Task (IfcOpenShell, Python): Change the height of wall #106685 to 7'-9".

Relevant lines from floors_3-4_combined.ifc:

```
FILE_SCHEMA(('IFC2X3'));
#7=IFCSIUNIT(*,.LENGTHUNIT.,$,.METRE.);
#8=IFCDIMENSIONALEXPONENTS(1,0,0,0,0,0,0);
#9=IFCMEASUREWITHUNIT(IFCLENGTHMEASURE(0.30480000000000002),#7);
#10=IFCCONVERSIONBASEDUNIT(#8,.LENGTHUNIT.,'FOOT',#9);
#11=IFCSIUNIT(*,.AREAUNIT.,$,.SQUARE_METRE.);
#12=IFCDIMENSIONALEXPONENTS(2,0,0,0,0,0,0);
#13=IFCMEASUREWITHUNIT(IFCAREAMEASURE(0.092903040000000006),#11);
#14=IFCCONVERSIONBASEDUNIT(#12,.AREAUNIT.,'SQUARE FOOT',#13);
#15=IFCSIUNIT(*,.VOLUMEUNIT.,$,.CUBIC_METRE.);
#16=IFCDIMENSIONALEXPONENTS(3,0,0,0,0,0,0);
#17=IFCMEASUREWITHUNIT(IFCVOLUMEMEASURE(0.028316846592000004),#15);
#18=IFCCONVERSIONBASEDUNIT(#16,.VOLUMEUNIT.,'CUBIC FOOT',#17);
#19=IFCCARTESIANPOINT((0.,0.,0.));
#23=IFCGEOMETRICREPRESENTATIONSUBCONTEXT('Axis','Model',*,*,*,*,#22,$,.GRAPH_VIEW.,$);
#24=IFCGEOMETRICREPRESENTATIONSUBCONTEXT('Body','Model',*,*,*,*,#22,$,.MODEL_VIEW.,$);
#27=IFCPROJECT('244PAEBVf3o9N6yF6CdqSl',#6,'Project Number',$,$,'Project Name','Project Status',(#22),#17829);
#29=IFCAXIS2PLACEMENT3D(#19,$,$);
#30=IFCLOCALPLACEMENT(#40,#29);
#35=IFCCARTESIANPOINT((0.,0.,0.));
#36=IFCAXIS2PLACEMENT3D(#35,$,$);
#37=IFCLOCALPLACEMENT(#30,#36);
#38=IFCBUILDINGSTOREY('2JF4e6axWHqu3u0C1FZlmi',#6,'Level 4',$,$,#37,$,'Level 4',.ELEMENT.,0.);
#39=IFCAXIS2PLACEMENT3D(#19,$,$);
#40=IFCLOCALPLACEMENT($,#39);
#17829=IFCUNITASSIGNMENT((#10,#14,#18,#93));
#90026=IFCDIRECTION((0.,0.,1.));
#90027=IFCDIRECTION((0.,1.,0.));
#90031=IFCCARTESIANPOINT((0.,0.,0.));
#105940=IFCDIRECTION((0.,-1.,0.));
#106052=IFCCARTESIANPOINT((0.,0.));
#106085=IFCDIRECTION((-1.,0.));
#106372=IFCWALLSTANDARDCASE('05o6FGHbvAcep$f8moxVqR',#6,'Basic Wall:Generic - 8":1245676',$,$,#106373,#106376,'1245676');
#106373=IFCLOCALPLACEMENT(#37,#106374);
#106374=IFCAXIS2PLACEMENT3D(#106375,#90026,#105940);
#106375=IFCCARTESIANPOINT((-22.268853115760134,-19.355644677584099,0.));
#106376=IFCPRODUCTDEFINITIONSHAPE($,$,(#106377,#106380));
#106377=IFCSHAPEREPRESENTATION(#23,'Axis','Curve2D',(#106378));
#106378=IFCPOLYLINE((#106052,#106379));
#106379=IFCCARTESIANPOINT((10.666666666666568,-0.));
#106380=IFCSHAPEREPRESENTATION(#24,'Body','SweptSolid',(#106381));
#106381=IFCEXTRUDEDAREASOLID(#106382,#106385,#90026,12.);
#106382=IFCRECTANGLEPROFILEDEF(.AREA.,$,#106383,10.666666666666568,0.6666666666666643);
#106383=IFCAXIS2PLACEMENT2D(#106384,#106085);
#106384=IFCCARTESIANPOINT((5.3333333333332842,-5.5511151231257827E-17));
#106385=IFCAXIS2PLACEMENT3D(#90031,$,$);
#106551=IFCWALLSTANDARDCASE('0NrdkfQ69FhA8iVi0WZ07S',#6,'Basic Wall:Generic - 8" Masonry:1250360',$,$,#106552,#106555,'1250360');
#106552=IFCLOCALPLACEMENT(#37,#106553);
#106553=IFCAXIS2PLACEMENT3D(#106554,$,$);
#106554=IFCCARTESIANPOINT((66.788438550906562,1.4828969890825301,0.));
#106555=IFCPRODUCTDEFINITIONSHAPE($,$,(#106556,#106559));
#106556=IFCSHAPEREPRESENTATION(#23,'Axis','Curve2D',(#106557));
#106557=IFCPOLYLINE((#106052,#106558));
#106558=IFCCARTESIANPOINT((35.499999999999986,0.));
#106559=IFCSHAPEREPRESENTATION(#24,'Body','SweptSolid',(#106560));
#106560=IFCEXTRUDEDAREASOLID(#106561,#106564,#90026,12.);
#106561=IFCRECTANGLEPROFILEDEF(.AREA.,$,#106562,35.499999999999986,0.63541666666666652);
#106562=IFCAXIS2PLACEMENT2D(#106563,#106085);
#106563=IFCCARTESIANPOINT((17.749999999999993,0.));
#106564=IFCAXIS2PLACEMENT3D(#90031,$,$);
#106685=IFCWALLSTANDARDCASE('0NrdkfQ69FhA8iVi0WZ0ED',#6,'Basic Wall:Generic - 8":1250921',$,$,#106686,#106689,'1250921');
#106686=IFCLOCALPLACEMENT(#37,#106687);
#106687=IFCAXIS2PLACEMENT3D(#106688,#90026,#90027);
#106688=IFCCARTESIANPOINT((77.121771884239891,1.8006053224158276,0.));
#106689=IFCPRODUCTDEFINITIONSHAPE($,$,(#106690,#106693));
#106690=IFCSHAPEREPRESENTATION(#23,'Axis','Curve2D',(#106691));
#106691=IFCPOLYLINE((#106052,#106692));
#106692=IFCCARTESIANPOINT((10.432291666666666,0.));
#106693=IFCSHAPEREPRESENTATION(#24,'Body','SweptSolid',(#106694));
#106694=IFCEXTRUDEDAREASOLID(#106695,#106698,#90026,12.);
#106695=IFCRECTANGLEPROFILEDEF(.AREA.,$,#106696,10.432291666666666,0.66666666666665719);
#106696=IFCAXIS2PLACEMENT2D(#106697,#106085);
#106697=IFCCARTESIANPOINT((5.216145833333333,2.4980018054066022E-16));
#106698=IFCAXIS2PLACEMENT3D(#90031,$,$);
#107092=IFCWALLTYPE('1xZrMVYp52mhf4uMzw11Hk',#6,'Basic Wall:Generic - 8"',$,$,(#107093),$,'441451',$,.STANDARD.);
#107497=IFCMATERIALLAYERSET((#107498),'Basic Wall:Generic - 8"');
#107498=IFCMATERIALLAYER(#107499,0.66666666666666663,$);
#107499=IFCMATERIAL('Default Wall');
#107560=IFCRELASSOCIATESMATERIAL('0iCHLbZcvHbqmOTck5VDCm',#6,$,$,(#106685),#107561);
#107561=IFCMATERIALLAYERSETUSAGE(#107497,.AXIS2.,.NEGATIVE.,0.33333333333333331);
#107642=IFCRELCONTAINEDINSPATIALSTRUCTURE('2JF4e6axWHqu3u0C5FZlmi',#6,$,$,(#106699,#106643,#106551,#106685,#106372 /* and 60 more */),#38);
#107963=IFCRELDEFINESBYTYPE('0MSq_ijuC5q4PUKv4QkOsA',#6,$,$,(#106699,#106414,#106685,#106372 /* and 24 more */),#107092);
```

```python
import ifcopenshell
import ifcopenshell.geom
import ifcopenshell.util.representation
import ifcopenshell.util.shape
import ifcopenshell.util.unit

model = ifcopenshell.open("floors_3-4_combined.ifc")
unit_scale = ifcopenshell.util.unit.calculate_unit_scale(model)
settings = ifcopenshell.geom.settings()


def volume(element):
    """Net volume in cubic metres, openings subtracted."""
    shape = ifcopenshell.geom.create_shape(settings, element)
    return ifcopenshell.util.shape.get_volume(shape.geometry)


wall = model.by_guid("0NrdkfQ69FhA8iVi0WZ0ED")
before = volume(wall)

body = ifcopenshell.util.representation.get_representation(wall, "Model", "Body")
solid = body.Items[0]
old_height = solid.Depth
solid.Depth = 93 * 0.0254 / unit_scale
after = volume(wall)

print(f"height {old_height:g} -> {solid.Depth:g}, volume {before:.3f} -> {after:.3f} m3")

model.write("floors_3-4_combined-out.ifc")
```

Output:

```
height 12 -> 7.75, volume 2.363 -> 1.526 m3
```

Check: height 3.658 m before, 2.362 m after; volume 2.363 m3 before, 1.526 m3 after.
